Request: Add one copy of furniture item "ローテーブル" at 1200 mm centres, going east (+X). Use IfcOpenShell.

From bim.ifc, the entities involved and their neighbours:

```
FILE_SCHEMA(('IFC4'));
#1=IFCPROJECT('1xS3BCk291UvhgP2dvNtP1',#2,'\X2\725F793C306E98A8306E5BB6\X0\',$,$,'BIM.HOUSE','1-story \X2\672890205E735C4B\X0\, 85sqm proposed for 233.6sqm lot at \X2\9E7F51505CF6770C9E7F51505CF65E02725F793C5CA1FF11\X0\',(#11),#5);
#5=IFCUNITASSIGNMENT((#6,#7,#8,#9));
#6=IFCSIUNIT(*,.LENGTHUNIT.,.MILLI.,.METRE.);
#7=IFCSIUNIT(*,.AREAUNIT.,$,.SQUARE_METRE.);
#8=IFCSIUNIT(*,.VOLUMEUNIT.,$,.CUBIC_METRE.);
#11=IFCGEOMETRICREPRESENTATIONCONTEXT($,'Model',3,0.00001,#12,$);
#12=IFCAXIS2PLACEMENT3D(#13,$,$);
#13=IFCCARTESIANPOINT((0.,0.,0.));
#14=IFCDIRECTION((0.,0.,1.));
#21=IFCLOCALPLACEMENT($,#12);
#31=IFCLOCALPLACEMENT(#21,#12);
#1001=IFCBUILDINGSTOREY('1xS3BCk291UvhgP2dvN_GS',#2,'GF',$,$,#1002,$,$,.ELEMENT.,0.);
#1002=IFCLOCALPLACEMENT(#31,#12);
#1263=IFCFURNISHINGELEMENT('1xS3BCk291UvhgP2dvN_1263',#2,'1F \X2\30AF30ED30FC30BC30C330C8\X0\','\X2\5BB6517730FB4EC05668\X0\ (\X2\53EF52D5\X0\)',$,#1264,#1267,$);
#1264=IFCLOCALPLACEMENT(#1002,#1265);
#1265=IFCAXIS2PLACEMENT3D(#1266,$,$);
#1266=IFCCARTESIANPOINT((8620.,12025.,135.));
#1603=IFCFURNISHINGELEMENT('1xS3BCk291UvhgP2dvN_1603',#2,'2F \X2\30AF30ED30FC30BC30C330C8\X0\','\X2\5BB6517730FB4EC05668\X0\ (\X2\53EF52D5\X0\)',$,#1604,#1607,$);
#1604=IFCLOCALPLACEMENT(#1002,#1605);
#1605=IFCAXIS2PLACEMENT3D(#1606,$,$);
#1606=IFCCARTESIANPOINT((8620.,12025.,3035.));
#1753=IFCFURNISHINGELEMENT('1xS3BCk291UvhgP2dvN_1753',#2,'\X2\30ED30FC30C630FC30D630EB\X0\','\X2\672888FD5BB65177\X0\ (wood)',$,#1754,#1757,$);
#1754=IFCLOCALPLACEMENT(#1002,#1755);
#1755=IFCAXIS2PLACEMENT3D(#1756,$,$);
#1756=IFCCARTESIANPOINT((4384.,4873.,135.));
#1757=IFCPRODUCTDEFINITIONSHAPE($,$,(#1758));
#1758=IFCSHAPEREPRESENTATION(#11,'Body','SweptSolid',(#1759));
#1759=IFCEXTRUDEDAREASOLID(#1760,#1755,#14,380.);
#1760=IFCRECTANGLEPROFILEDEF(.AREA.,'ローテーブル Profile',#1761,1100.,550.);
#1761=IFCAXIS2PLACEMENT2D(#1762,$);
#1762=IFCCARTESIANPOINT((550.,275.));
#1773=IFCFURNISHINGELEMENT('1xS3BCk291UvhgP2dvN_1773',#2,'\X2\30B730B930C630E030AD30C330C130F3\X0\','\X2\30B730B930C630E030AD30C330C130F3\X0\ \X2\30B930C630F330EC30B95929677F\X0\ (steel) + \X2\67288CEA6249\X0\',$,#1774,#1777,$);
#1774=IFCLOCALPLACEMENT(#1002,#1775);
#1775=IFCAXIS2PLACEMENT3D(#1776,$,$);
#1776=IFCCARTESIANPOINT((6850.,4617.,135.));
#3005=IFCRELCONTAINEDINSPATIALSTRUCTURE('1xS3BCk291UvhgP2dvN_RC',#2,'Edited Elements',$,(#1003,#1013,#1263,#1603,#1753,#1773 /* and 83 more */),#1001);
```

```python
import numpy as np
import ifcopenshell
import ifcopenshell.api.geometry
import ifcopenshell.api.root
import ifcopenshell.util.element
import ifcopenshell.util.placement
import ifcopenshell.util.unit

model = ifcopenshell.open("bim.ifc")
unit_scale = ifcopenshell.util.unit.calculate_unit_scale(model)


def reuse_history(source, copy):
    """copy_class also copies each property set's owner history, people and application; keep the originals."""
    for rel in copy.IsDefinedBy:
        if rel.is_a("IfcRelDefinesByProperties") and (history := rel.RelatingPropertyDefinition.OwnerHistory):
            rel.RelatingPropertyDefinition.OwnerHistory = source.OwnerHistory
            ifcopenshell.util.element.remove_deep2(model, history)


source = model.by_guid("1xS3BCk291UvhgP2dvN_1753")
base = ifcopenshell.util.placement.get_local_placement(source.ObjectPlacement)
step = np.array([1.0, 0.0, 0.0]) * 1.2 / unit_scale

for i in range(1, 2):
    copy = ifcopenshell.api.root.copy_class(model, product=source)
    copy.Representation = ifcopenshell.util.element.copy_deep(
        model, source.Representation, exclude=["IfcGeometricRepresentationContext", "IfcRepresentationMap"]
    )
    reuse_history(source, copy)
    matrix = base.copy()
    matrix[:3, 3] += i * step
    print("added at", matrix[:3, 3].round(3) + 0.0)
    ifcopenshell.api.geometry.edit_object_placement(model, product=copy, matrix=matrix, is_si=False)

model.write("bim_updated.ifc")
```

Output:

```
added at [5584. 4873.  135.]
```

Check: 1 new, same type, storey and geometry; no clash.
